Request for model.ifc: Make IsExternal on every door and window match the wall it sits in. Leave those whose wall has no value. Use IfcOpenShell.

First a look at what the model holds.

```python
import ifcopenshell
import ifcopenshell.util.element

model = ifcopenshell.open("model.ifc")
print(model.schema)
seen = {}
for e in model.by_type("IfcDoor") + model.by_type("IfcWindow"):
    if not e.FillsVoids:
        continue
    host = e.FillsVoids[0].RelatingOpeningElement.VoidsElements[0].RelatingBuildingElement
    own = ifcopenshell.util.element.get_pset(e, f"Pset_{e.is_a()[3:].removesuffix('StandardCase')}Common", "IsExternal")
    wall = ifcopenshell.util.element.get_pset(host, "Pset_WallCommon", "IsExternal")
    seen[e.is_a(), own, wall] = seen.get((e.is_a(), own, wall), 0) + 1
for (cls, own, wall), count in sorted(seen.items(), key=str):
    print(count, cls, "IsExternal:", own, "| host wall:", wall)
```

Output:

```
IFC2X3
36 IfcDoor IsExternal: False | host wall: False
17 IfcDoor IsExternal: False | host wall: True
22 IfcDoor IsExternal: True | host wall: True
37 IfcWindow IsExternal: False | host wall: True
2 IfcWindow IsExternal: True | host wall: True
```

```python
import ifcopenshell
import ifcopenshell.api.pset
import ifcopenshell.util.element

model = ifcopenshell.open("model.ifc")

count = 0
for ifc_class, pset_name in (("IfcDoor", "Pset_DoorCommon"), ("IfcWindow", "Pset_WindowCommon")):
    for e in model.by_type(ifc_class):
        if not e.FillsVoids:
            continue
        host = e.FillsVoids[0].RelatingOpeningElement.VoidsElements[0].RelatingBuildingElement
        external = ifcopenshell.util.element.get_pset(host, "Pset_WallCommon", "IsExternal")
        if external is None or ifcopenshell.util.element.get_pset(e, pset_name, "IsExternal") == external:
            continue
        pset = ifcopenshell.api.pset.add_pset(model, product=e, name=pset_name)
        ifcopenshell.api.pset.edit_pset(model, pset=pset, properties={"IsExternal": external})
        count += 1

print(count, "updated")

model.write("model_edited.ifc")
```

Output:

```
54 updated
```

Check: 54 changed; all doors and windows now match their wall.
